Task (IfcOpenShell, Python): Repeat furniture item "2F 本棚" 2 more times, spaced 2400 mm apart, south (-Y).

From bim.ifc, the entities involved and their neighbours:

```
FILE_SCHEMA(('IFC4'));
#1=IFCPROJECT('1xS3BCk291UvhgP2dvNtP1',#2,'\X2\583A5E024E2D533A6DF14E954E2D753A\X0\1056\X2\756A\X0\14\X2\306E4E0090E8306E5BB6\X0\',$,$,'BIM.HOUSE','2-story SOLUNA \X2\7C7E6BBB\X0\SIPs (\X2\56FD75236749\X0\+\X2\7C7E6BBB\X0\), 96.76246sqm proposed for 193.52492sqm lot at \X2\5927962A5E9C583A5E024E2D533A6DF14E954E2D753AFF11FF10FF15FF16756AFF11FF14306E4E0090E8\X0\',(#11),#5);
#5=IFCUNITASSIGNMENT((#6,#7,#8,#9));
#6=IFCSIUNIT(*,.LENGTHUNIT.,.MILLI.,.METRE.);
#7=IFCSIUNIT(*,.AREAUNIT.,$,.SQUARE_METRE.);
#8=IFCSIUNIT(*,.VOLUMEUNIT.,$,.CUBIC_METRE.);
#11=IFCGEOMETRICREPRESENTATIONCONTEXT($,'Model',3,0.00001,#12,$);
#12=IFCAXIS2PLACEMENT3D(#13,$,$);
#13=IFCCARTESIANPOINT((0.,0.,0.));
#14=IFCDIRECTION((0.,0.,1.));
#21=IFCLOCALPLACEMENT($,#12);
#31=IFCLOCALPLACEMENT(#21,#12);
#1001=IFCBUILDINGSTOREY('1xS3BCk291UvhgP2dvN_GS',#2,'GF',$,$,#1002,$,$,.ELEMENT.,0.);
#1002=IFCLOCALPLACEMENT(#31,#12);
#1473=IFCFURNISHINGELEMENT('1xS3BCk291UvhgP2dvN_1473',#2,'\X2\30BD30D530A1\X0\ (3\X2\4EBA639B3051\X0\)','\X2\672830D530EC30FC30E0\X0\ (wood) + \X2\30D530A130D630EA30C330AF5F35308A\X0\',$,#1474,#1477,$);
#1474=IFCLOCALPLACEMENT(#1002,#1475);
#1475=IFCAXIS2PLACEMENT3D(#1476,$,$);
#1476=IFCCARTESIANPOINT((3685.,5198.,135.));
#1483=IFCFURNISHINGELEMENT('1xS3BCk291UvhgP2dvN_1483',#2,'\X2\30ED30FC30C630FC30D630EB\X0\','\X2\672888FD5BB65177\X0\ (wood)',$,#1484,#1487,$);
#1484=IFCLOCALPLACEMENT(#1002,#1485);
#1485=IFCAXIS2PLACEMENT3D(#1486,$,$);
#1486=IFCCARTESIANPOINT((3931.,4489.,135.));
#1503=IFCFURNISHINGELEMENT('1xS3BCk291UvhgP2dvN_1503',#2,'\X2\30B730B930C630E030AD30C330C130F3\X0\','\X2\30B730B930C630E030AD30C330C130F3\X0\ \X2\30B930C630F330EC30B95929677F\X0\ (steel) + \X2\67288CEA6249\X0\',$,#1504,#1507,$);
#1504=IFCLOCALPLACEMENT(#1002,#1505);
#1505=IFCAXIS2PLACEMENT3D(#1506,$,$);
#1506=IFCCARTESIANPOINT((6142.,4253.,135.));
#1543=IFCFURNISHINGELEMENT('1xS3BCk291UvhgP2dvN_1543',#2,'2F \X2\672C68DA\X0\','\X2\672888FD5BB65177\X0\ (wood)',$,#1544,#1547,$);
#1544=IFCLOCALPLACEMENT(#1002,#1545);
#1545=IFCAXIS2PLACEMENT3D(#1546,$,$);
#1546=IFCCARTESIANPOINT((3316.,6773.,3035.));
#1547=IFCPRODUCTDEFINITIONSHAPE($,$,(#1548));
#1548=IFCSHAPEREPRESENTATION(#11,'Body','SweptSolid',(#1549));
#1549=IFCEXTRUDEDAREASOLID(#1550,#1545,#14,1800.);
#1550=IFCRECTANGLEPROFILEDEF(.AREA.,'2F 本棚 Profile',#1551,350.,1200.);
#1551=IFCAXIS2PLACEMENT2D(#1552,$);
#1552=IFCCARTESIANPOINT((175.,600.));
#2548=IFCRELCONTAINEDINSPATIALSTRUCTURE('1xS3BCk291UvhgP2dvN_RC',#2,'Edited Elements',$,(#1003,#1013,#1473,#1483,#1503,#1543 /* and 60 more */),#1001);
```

```python
import numpy as np
import ifcopenshell
import ifcopenshell.api.geometry
import ifcopenshell.api.root
import ifcopenshell.util.element
import ifcopenshell.util.placement

model = ifcopenshell.open("bim.ifc")


def reuse_history(source, copy):
    """copy_class also copies each property set's owner history, people and application; keep the originals."""
    for rel in copy.IsDefinedBy:
        if rel.is_a("IfcRelDefinesByProperties") and (history := rel.RelatingPropertyDefinition.OwnerHistory):
            rel.RelatingPropertyDefinition.OwnerHistory = source.OwnerHistory
            ifcopenshell.util.element.remove_deep2(model, history)


source = model.by_guid("1xS3BCk291UvhgP2dvN_1543")
base = ifcopenshell.util.placement.get_local_placement(source.ObjectPlacement)
step = np.array([0.0, -1.0, 0.0]) * 2400.0

for i in range(1, 3):
    copy = ifcopenshell.api.root.copy_class(model, product=source)
    copy.Representation = ifcopenshell.util.element.copy_deep(
        model, source.Representation, exclude=["IfcGeometricRepresentationContext", "IfcRepresentationMap"]
    )
    reuse_history(source, copy)
    matrix = base.copy()
    matrix[:3, 3] += i * step
    print("added at", matrix[:3, 3].round(3) + 0.0)
    ifcopenshell.api.geometry.edit_object_placement(model, product=copy, matrix=matrix, is_si=False)

model.write("bim_updated.ifc")
```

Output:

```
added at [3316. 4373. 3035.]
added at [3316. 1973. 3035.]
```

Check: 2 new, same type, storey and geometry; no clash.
